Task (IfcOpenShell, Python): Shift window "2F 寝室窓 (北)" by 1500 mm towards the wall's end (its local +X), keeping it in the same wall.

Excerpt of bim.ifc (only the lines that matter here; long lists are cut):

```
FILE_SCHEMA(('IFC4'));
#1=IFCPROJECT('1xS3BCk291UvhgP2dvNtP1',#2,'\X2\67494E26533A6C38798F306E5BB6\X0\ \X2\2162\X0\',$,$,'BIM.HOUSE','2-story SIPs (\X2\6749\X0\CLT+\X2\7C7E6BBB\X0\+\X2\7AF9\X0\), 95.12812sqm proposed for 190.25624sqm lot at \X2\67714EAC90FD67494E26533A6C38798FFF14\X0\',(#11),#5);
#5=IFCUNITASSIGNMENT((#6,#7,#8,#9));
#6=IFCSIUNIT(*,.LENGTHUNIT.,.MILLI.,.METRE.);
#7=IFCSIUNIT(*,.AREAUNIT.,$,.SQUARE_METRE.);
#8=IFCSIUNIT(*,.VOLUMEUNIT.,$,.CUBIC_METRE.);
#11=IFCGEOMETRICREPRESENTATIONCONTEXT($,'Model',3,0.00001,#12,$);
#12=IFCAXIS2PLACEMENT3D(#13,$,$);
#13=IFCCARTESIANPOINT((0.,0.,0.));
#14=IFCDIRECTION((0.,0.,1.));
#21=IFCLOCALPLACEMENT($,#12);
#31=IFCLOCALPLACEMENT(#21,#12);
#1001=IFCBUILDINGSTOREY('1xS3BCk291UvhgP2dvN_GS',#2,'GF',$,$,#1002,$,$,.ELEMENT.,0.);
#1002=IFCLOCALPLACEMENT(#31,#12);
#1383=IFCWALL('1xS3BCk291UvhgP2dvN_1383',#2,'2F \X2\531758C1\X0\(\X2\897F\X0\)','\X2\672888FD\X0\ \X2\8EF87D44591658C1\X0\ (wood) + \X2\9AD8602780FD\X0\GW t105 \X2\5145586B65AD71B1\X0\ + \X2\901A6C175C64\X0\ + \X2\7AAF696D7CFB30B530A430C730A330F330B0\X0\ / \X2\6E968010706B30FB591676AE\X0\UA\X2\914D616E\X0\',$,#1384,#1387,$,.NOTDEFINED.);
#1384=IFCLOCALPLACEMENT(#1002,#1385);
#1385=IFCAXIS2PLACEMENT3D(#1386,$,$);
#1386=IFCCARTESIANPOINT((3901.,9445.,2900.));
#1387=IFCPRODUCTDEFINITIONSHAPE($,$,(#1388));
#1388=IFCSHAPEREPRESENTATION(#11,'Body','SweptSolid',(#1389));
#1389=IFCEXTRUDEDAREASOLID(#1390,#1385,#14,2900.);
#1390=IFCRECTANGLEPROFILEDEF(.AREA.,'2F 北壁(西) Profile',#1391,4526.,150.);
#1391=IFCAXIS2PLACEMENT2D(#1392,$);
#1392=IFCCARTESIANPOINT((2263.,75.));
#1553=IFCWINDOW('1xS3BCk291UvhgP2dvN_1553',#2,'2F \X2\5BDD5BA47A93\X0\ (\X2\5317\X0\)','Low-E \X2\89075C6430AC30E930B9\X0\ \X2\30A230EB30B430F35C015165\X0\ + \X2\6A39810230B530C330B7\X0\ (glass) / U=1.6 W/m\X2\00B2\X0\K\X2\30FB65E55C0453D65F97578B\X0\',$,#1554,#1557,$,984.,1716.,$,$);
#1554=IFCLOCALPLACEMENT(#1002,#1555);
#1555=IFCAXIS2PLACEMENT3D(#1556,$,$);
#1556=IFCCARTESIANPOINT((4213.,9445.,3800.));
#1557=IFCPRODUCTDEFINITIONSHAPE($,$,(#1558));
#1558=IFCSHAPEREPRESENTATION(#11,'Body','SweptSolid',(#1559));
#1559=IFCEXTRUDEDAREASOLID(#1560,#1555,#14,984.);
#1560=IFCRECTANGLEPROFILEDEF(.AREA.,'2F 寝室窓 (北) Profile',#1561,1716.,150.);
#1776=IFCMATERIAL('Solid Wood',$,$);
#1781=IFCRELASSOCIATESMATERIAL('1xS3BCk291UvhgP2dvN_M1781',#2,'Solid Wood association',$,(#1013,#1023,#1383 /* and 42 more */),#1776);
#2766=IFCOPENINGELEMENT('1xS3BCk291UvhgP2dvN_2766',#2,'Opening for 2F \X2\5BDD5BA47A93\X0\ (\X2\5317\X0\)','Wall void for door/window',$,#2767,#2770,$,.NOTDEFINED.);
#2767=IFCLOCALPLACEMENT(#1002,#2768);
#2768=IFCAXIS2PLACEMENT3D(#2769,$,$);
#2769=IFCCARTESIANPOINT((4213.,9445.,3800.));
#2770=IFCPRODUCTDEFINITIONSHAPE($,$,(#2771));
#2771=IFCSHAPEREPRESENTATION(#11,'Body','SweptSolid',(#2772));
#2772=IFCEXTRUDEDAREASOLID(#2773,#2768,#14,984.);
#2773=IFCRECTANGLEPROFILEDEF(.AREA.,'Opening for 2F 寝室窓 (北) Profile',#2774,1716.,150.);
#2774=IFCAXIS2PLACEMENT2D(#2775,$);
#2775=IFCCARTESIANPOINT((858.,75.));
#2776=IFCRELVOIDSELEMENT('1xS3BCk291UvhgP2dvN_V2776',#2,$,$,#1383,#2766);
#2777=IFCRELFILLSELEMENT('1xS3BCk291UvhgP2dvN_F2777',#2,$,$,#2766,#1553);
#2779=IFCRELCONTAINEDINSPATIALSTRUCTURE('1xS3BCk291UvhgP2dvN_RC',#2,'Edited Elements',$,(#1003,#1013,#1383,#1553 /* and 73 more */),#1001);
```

```python
import ifcopenshell
import ifcopenshell.api.geometry
import ifcopenshell.util.placement
import ifcopenshell.util.unit

model = ifcopenshell.open("bim.ifc")
unit_scale = ifcopenshell.util.unit.calculate_unit_scale(model)

window = model.by_id(1553)
opening = window.FillsVoids[0].RelatingOpeningElement
wall = opening.VoidsElements[0].RelatingBuildingElement

wall_matrix = ifcopenshell.util.placement.get_local_placement(wall.ObjectPlacement)
shift = wall_matrix[:3, 0] * 1.5 / unit_scale
before = ifcopenshell.util.placement.get_local_placement(window.ObjectPlacement)[:3, 3].copy()

# The window is not placed relative to its opening, so move both.
for product in (opening, window):
    matrix = ifcopenshell.util.placement.get_local_placement(product.ObjectPlacement)
    matrix[:3, 3] += shift
    ifcopenshell.api.geometry.edit_object_placement(model, product=product, matrix=matrix, is_si=False)

after = ifcopenshell.util.placement.get_local_placement(window.ObjectPlacement)[:3, 3]
print("window moved by", (after - before).round(3) + 0.0)

model.write("bim_v2.ifc")
```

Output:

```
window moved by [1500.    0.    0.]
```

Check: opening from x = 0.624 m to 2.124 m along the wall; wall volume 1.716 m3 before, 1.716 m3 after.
